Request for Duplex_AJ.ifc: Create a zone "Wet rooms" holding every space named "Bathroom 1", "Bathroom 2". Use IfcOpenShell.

First a look at what the model holds.

```python
import ifcopenshell

model = ifcopenshell.open("Duplex_AJ.ifc")
print(model.schema)
seen = {}
for space in model.by_type("IfcSpace"):
    seen[space.LongName] = seen.get(space.LongName, 0) + 1
for name, count in sorted(seen.items(), key=str):
    print(count, "x", name)
print("zones:", [z.Name for z in model.by_type("IfcZone")][:20])
```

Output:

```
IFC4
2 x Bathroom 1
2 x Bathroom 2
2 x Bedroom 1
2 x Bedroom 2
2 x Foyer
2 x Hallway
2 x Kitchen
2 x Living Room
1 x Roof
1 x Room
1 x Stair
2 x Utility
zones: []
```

```python
import ifcopenshell
import ifcopenshell.api.group
import ifcopenshell.api.root

model = ifcopenshell.open("Duplex_AJ.ifc")

names = {"Bathroom 1", "Bathroom 2"}
spaces = [s for s in model.by_type("IfcSpace") if s.LongName in names]

zone = ifcopenshell.api.root.create_entity(model, ifc_class="IfcZone", name="Wet rooms")
ifcopenshell.api.group.assign_group(model, products=spaces, group=zone)
print(len(spaces), "spaces in", zone.Name)

model.write("Duplex_AJ_rev.ifc")
```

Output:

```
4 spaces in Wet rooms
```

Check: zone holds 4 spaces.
